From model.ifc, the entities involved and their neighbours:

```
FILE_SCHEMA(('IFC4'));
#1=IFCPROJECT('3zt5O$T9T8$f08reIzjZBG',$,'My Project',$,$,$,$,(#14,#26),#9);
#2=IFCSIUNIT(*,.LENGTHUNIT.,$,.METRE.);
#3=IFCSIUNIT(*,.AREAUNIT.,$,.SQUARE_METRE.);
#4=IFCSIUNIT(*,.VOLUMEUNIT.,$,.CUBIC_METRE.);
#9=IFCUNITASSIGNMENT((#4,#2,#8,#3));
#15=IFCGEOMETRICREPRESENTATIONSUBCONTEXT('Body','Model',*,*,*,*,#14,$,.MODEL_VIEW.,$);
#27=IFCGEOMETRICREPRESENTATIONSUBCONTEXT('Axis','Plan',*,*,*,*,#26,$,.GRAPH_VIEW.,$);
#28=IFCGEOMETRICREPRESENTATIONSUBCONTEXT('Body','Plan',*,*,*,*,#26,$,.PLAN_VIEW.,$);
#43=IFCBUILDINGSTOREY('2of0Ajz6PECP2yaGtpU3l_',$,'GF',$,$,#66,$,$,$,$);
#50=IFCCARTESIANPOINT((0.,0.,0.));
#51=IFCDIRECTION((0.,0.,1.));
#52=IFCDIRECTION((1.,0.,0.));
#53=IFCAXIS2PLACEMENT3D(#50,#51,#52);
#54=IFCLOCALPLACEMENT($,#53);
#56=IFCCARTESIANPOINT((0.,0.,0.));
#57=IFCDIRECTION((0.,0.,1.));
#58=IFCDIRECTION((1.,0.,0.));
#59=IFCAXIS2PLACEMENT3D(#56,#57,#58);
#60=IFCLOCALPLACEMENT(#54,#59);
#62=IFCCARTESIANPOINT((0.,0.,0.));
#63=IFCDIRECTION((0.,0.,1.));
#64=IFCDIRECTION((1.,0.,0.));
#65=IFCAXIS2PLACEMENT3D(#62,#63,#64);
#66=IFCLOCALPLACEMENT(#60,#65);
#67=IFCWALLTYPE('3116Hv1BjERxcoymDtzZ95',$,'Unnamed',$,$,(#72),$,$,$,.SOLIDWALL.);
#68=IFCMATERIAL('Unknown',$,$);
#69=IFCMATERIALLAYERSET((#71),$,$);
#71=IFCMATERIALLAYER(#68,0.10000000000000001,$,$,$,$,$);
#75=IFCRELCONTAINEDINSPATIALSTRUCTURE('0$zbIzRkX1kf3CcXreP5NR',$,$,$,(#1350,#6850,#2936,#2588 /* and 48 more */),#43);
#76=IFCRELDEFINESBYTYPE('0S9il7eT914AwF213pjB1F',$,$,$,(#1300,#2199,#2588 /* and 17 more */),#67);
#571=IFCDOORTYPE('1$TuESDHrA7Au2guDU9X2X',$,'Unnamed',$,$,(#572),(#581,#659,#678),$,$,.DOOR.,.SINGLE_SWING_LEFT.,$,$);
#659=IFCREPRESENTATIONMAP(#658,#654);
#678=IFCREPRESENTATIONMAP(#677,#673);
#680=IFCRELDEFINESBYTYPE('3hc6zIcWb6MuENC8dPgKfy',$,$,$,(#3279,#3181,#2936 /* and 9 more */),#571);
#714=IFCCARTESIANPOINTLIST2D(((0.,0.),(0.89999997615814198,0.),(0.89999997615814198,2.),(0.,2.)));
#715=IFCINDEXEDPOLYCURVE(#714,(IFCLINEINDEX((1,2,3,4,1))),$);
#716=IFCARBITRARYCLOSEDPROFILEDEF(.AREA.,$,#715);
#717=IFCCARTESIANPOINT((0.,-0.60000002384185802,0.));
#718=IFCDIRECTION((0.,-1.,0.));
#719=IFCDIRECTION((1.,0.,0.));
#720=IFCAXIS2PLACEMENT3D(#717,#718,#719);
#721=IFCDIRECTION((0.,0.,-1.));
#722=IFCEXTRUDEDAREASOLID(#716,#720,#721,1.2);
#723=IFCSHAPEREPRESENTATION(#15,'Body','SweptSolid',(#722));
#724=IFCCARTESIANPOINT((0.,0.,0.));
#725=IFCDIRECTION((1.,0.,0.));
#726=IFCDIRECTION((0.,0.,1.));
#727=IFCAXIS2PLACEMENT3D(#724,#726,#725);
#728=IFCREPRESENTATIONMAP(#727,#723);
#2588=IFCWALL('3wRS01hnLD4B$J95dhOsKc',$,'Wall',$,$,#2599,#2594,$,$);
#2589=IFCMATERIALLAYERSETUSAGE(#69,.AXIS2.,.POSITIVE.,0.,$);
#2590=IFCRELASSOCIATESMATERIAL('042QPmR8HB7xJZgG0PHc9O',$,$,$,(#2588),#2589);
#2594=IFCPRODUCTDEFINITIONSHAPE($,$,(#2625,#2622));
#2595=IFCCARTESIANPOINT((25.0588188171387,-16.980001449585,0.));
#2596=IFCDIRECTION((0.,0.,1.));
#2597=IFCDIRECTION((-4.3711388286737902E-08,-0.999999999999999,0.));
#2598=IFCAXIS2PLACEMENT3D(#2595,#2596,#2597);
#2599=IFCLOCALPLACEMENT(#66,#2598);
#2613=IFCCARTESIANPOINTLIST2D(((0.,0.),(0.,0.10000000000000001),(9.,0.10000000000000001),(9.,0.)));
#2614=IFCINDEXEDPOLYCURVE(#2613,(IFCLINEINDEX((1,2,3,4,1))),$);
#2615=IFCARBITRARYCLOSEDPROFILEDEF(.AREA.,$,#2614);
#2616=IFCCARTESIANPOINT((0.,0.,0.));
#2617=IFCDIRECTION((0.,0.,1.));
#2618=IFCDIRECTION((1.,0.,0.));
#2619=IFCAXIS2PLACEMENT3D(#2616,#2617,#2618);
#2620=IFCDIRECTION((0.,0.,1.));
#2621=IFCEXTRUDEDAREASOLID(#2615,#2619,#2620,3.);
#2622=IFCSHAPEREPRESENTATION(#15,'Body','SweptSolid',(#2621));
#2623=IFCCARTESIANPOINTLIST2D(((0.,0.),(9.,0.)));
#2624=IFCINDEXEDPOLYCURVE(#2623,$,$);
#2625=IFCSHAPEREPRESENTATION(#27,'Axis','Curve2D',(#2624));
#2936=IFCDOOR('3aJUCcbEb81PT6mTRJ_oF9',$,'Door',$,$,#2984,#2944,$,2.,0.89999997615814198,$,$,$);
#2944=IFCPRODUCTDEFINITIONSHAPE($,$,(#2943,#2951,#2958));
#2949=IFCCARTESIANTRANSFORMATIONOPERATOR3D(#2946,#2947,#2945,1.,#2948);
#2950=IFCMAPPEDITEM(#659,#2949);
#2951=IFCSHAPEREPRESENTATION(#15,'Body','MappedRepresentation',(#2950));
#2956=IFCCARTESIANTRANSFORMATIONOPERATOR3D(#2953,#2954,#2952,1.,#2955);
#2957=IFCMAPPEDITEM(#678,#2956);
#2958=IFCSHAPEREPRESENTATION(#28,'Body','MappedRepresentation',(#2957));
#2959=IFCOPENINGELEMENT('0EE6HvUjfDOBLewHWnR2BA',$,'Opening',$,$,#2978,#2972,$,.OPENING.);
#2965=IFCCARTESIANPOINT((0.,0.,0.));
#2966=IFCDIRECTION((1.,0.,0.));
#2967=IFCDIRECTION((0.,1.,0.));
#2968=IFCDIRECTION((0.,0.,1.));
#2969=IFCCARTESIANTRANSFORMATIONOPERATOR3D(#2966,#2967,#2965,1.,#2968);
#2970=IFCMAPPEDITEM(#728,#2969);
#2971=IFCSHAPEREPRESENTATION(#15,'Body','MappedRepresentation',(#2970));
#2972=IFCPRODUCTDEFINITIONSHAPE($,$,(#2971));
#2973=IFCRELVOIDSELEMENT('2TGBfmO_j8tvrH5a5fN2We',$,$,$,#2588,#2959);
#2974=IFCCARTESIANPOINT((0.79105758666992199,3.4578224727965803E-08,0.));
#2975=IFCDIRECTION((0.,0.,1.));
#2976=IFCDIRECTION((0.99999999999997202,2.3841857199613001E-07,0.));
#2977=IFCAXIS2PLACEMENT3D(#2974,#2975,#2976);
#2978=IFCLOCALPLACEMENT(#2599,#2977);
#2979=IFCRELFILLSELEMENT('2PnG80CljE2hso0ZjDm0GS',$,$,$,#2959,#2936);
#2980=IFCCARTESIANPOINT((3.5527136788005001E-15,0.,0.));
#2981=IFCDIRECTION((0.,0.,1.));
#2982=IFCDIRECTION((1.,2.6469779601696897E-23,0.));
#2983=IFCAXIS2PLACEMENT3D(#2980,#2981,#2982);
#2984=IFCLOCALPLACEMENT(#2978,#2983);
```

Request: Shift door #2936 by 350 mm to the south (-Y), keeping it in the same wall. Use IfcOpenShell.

```python
import ifcopenshell
import ifcopenshell.api.geometry
import ifcopenshell.util.placement
import ifcopenshell.util.unit

model = ifcopenshell.open("model.ifc")
unit_scale = ifcopenshell.util.unit.calculate_unit_scale(model)

door = model.by_guid("3aJUCcbEb81PT6mTRJ_oF9")
opening = door.FillsVoids[0].RelatingOpeningElement
wall = opening.VoidsElements[0].RelatingBuildingElement

wall_matrix = ifcopenshell.util.placement.get_local_placement(wall.ObjectPlacement)
shift = wall_matrix[:3, 0] * 0.35 / unit_scale
before = ifcopenshell.util.placement.get_local_placement(door.ObjectPlacement)[:3, 3].copy()

# The door is placed relative to its opening, so it follows when the opening moves.
matrix = ifcopenshell.util.placement.get_local_placement(opening.ObjectPlacement)
matrix[:3, 3] += shift
ifcopenshell.api.geometry.edit_object_placement(
    model, product=opening, matrix=matrix, is_si=False, should_transform_children=True
)

after = ifcopenshell.util.placement.get_local_placement(door.ObjectPlacement)[:3, 3]
print("door moved by", (after - before).round(3) + 0.0)

model.write("model_rev.ifc")
```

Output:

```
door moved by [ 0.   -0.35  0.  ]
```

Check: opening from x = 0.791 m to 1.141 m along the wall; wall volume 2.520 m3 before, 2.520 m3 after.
